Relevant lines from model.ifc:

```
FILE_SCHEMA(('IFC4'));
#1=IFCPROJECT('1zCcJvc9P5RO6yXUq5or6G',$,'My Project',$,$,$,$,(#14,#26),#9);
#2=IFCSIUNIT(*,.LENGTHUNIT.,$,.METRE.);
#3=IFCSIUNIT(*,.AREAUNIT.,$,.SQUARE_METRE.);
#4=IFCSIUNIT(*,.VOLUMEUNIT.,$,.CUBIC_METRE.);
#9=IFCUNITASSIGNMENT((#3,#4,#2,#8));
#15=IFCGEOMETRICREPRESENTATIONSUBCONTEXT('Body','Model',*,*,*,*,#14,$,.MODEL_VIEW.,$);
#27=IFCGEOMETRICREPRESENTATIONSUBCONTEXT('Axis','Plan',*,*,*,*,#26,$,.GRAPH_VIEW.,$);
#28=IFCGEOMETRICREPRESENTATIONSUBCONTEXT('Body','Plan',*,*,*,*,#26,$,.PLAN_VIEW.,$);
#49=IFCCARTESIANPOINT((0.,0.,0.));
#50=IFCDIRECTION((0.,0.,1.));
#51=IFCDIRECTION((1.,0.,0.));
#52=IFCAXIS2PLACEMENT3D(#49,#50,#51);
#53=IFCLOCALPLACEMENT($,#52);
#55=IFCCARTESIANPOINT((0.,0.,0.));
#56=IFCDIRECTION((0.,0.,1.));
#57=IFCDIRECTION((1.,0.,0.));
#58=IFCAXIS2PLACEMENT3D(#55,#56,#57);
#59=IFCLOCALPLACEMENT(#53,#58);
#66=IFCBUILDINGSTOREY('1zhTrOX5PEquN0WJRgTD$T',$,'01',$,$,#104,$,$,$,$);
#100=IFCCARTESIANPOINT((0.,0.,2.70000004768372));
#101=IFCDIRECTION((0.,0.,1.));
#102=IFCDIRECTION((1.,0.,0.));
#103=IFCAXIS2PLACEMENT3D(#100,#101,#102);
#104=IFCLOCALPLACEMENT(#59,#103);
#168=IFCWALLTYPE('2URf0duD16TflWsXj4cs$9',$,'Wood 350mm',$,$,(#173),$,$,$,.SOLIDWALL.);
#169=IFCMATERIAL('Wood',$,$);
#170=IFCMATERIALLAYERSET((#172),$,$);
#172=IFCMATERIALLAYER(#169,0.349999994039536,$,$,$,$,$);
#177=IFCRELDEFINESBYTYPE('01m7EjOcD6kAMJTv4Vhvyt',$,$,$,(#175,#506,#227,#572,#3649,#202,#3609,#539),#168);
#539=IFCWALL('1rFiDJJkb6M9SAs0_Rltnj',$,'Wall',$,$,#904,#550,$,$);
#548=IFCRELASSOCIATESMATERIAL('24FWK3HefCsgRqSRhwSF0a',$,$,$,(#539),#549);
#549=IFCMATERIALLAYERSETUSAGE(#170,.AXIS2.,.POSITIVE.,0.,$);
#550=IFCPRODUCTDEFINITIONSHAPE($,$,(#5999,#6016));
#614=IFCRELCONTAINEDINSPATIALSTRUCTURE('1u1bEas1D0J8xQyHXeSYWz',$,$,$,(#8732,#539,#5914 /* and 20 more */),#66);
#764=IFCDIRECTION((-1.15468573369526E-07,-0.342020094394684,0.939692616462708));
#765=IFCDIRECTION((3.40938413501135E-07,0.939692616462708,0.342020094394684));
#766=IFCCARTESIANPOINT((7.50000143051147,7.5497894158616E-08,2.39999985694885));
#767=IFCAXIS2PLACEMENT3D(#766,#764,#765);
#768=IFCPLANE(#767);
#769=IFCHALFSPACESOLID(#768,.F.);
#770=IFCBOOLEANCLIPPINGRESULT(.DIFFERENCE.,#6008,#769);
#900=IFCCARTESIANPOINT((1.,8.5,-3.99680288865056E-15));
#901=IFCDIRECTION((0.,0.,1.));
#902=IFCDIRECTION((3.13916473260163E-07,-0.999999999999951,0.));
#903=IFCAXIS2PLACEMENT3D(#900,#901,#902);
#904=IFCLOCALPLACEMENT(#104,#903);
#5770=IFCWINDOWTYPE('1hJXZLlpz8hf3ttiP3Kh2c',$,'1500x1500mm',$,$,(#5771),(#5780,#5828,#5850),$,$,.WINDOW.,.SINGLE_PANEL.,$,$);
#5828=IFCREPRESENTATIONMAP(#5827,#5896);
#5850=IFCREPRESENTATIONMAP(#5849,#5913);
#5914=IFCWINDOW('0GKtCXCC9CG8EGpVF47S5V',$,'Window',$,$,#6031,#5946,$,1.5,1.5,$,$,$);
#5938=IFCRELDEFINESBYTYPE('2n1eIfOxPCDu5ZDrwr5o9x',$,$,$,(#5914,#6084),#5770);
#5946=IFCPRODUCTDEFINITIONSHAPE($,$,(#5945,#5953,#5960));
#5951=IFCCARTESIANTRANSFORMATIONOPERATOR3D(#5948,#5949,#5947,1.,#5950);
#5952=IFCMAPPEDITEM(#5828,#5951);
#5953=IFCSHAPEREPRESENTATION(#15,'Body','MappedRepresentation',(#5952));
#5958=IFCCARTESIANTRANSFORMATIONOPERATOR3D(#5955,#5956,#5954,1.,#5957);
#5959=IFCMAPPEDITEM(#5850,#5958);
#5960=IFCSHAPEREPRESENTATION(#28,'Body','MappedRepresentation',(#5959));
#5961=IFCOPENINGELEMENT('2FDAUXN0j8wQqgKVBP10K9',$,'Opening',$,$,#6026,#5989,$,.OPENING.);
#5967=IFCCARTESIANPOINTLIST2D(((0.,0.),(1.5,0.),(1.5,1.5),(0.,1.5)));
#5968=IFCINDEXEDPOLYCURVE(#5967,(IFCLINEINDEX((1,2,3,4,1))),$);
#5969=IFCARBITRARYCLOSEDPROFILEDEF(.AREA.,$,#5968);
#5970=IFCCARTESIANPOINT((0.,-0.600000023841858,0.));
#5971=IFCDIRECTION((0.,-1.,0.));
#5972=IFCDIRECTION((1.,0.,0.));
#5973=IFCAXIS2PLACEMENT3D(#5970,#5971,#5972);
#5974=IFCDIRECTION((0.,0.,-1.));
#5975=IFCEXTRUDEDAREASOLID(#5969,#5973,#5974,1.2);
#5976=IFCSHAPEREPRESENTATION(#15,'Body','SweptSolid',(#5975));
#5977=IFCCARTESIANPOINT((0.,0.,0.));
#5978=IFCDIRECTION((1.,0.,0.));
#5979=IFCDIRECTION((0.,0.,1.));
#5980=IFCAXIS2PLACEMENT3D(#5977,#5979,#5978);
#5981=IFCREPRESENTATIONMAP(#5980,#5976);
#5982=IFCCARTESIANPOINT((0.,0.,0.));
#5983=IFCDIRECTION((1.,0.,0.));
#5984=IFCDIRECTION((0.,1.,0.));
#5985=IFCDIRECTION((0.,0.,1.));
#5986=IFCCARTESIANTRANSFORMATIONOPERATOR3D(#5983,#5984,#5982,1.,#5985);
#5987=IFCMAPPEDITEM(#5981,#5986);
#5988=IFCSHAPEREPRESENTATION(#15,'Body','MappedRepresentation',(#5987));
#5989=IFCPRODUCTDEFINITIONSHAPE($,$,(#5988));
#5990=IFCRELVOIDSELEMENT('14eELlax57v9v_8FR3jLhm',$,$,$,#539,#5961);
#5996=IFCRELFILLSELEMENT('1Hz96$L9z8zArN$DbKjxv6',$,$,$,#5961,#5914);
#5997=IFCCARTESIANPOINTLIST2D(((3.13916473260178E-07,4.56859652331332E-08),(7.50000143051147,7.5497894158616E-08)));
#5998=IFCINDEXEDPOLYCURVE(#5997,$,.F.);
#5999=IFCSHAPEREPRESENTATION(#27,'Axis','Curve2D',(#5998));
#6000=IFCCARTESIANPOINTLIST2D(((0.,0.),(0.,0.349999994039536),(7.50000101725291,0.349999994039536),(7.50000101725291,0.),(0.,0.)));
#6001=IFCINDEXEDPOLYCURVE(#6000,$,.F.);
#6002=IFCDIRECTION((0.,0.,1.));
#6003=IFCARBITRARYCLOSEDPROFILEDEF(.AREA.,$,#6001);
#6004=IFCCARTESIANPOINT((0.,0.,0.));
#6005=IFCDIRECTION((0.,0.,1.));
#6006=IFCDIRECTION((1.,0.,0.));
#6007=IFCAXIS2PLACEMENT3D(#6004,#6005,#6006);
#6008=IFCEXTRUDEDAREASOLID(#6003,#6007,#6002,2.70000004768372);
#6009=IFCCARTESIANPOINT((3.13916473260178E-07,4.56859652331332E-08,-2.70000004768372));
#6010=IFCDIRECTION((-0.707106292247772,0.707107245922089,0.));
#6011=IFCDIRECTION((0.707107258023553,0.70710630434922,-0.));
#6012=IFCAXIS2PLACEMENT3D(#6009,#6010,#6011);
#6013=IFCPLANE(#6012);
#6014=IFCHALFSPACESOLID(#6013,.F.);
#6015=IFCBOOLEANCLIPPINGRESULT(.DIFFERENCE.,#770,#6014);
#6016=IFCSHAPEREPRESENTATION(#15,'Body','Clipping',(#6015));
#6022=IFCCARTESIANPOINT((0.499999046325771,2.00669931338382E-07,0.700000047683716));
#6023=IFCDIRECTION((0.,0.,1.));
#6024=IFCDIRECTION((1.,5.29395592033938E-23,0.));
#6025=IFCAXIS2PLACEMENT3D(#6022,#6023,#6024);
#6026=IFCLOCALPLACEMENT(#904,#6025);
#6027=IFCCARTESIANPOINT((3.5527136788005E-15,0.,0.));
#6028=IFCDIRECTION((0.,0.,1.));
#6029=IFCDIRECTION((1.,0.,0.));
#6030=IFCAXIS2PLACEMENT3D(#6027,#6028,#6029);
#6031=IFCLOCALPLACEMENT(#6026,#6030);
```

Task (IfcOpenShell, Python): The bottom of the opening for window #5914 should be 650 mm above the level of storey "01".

```python
import numpy as np
import ifcopenshell
import ifcopenshell.api.geometry
import ifcopenshell.geom
import ifcopenshell.util.element
import ifcopenshell.util.placement
import ifcopenshell.util.shape
import ifcopenshell.util.unit

model = ifcopenshell.open("model.ifc")
unit_scale = ifcopenshell.util.unit.calculate_unit_scale(model)

window = model.by_guid("0GKtCXCC9CG8EGpVF47S5V")
opening = window.FillsVoids[0].RelatingOpeningElement
storey = ifcopenshell.util.element.get_container(window, ifc_class="IfcBuildingStorey")
level = ifcopenshell.util.placement.get_local_placement(storey.ObjectPlacement)[2, 3]

# The opening's origin need not be at the sill, so measure its lowest point.
shape = ifcopenshell.geom.create_shape(ifcopenshell.geom.settings(), opening)
bottom = ifcopenshell.util.shape.get_shape_bottom_elevation(shape, shape.geometry) / unit_scale
dz = level + 0.65 / unit_scale - bottom

shift = np.array([0.0, 0.0, dz])
# The window is placed relative to its opening, so it follows when the opening moves.
matrix = ifcopenshell.util.placement.get_local_placement(opening.ObjectPlacement)
matrix[:3, 3] += shift
ifcopenshell.api.geometry.edit_object_placement(
    model, product=opening, matrix=matrix, is_si=False, should_transform_children=True
)

print(f"moved by {dz * unit_scale:+.3f} m")

model.write("model_edited.ifc")
```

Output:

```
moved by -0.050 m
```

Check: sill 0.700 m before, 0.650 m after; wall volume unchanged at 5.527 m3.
